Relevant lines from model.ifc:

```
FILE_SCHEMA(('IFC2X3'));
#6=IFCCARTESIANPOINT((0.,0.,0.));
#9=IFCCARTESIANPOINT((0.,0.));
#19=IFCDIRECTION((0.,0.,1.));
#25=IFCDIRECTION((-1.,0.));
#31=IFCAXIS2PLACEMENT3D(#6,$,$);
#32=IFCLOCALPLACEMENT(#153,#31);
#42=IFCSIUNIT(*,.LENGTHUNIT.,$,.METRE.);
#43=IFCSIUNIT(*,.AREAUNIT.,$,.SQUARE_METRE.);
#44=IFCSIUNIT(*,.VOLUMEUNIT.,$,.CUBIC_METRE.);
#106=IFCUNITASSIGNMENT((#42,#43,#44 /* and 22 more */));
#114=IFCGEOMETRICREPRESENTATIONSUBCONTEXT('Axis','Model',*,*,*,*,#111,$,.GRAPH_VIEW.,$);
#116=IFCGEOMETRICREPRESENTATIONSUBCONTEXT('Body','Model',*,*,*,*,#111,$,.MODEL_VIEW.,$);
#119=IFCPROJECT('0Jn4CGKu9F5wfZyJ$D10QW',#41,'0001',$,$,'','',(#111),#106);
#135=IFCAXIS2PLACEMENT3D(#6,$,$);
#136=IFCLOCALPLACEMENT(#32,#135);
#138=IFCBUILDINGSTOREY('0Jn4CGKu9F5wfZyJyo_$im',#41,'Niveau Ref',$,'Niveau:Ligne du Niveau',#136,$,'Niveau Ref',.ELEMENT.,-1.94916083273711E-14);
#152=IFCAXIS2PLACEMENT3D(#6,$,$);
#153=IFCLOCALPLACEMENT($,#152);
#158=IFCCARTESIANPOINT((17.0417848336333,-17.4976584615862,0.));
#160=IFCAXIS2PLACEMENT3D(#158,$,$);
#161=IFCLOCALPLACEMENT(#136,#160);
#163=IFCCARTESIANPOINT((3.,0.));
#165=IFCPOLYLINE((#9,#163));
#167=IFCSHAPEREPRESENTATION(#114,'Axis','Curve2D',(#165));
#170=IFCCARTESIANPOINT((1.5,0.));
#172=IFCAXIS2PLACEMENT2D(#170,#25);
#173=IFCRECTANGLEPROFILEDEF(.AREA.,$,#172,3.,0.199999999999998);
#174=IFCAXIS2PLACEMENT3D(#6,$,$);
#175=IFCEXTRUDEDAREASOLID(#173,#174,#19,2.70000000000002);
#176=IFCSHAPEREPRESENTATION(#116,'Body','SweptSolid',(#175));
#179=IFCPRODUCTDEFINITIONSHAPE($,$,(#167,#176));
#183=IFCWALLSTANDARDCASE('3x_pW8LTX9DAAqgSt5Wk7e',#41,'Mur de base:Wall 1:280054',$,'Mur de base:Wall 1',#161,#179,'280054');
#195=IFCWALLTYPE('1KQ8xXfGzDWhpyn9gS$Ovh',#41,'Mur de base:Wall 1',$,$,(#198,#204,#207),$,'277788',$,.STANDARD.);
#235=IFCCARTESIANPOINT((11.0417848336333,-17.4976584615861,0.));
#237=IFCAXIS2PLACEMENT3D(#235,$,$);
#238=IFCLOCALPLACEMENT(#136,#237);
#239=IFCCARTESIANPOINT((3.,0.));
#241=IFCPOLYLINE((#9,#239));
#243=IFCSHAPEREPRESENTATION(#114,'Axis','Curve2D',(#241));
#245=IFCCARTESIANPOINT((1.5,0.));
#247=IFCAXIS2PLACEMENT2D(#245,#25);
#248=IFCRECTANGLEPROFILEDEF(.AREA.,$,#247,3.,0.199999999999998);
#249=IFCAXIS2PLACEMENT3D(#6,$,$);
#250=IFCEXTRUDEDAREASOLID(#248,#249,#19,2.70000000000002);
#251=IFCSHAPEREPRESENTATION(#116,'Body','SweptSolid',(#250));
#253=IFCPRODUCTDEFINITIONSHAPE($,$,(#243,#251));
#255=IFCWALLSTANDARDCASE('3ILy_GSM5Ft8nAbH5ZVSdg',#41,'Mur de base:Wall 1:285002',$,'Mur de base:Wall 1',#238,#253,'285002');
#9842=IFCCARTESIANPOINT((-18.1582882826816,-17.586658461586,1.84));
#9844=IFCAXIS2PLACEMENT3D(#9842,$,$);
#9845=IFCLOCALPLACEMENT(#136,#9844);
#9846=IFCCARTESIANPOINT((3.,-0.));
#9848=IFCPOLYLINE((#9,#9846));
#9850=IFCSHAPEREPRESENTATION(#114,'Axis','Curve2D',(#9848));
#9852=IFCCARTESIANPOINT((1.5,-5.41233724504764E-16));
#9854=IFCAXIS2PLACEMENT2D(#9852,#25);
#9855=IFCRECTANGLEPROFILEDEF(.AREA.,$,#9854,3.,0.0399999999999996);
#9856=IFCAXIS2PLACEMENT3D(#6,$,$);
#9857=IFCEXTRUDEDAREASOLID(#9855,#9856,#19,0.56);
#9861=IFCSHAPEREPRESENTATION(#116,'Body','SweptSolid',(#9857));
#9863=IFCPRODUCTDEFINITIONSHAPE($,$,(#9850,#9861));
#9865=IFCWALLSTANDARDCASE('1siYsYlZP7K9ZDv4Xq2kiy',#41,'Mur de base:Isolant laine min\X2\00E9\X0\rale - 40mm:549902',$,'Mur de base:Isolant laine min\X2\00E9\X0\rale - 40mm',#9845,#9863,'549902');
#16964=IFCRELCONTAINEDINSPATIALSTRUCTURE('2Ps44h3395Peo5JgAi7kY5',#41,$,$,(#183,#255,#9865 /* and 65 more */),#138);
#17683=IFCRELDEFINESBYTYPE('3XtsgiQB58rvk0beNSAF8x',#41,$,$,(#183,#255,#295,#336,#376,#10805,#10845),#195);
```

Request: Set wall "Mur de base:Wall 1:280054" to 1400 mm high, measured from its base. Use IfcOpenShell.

```python
import ifcopenshell
import ifcopenshell.geom
import ifcopenshell.util.representation
import ifcopenshell.util.shape

model = ifcopenshell.open("model.ifc")
settings = ifcopenshell.geom.settings()


def volume(element):
    """Net volume in cubic metres, openings subtracted."""
    shape = ifcopenshell.geom.create_shape(settings, element)
    return ifcopenshell.util.shape.get_volume(shape.geometry)


wall = model.by_guid("3x_pW8LTX9DAAqgSt5Wk7e")
before = volume(wall)

body = ifcopenshell.util.representation.get_representation(wall, "Model", "Body")
solid = body.Items[0]
old_height = solid.Depth
solid.Depth = 1.4
after = volume(wall)

print(f"height {old_height:g} -> {solid.Depth:g}, volume {before:.3f} -> {after:.3f} m3")

model.write("model_updated.ifc")
```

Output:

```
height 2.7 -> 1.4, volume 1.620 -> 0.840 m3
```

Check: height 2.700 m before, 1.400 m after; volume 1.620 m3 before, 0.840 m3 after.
